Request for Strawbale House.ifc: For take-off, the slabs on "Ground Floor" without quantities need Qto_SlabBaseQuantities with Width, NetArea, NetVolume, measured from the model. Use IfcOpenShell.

First a look at what the model holds.

```python
import ifcopenshell
import ifcopenshell.util.element
import ifcopenshell.util.unit

model = ifcopenshell.open("Strawbale House.ifc")
print(model.schema)
for unit_type in ("LENGTHUNIT", "AREAUNIT", "VOLUMEUNIT"):
    print(unit_type, ifcopenshell.util.unit.calculate_unit_scale(model, unit_type))
storey = next(s for s in model.by_type("IfcBuildingStorey") if s.Name == "Ground Floor")
slabs = [e for e in ifcopenshell.util.element.get_decomposition(storey) if e.is_a("IfcSlab")]
for e in sorted(slabs, key=lambda e: e.id()):
    print(e.id(), e.is_a(), e.Name, list(ifcopenshell.util.element.get_psets(e, qtos_only=True)), sep=" | ")
```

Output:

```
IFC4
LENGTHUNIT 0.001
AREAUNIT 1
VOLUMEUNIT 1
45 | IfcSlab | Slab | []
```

```python
import ifcopenshell
import ifcopenshell.api.pset
import ifcopenshell.geom
import ifcopenshell.util.element
import ifcopenshell.util.shape
import ifcopenshell.util.unit

model = ifcopenshell.open("Strawbale House.ifc")
unit_scale = ifcopenshell.util.unit.calculate_unit_scale(model)
area_scale = ifcopenshell.util.unit.calculate_unit_scale(model, "AREAUNIT")
volume_scale = ifcopenshell.util.unit.calculate_unit_scale(model, "VOLUMEUNIT")
settings = ifcopenshell.geom.settings()

storey = next(s for s in model.by_type("IfcBuildingStorey") if s.Name == "Ground Floor")
slabs = [e for e in ifcopenshell.util.element.get_decomposition(storey) if e.is_a("IfcSlab")]

for e in sorted(slabs, key=lambda e: e.id()):
    if ifcopenshell.util.element.get_psets(e, qtos_only=True, should_inherit=False):
        continue
    # Geometry comes back in metres, in the element's own axes.
    shape = ifcopenshell.geom.create_shape(settings, e)
    values = {
        "Width": ifcopenshell.util.shape.get_z(shape.geometry) / unit_scale,
        "NetArea": ifcopenshell.util.shape.get_footprint_area(shape.geometry) / area_scale,
        "NetVolume": ifcopenshell.util.shape.get_volume(shape.geometry) / volume_scale,
    }
    qto = ifcopenshell.api.pset.add_qto(model, product=e, name="Qto_SlabBaseQuantities")
    ifcopenshell.api.pset.edit_qto(model, qto=qto, properties=values)
    print(e.id(), {k: round(v, 3) for k, v in values.items()})

model.write("Strawbale House_edited.ifc")
```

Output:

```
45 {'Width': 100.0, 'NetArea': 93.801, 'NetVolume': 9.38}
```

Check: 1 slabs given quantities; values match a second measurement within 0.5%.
